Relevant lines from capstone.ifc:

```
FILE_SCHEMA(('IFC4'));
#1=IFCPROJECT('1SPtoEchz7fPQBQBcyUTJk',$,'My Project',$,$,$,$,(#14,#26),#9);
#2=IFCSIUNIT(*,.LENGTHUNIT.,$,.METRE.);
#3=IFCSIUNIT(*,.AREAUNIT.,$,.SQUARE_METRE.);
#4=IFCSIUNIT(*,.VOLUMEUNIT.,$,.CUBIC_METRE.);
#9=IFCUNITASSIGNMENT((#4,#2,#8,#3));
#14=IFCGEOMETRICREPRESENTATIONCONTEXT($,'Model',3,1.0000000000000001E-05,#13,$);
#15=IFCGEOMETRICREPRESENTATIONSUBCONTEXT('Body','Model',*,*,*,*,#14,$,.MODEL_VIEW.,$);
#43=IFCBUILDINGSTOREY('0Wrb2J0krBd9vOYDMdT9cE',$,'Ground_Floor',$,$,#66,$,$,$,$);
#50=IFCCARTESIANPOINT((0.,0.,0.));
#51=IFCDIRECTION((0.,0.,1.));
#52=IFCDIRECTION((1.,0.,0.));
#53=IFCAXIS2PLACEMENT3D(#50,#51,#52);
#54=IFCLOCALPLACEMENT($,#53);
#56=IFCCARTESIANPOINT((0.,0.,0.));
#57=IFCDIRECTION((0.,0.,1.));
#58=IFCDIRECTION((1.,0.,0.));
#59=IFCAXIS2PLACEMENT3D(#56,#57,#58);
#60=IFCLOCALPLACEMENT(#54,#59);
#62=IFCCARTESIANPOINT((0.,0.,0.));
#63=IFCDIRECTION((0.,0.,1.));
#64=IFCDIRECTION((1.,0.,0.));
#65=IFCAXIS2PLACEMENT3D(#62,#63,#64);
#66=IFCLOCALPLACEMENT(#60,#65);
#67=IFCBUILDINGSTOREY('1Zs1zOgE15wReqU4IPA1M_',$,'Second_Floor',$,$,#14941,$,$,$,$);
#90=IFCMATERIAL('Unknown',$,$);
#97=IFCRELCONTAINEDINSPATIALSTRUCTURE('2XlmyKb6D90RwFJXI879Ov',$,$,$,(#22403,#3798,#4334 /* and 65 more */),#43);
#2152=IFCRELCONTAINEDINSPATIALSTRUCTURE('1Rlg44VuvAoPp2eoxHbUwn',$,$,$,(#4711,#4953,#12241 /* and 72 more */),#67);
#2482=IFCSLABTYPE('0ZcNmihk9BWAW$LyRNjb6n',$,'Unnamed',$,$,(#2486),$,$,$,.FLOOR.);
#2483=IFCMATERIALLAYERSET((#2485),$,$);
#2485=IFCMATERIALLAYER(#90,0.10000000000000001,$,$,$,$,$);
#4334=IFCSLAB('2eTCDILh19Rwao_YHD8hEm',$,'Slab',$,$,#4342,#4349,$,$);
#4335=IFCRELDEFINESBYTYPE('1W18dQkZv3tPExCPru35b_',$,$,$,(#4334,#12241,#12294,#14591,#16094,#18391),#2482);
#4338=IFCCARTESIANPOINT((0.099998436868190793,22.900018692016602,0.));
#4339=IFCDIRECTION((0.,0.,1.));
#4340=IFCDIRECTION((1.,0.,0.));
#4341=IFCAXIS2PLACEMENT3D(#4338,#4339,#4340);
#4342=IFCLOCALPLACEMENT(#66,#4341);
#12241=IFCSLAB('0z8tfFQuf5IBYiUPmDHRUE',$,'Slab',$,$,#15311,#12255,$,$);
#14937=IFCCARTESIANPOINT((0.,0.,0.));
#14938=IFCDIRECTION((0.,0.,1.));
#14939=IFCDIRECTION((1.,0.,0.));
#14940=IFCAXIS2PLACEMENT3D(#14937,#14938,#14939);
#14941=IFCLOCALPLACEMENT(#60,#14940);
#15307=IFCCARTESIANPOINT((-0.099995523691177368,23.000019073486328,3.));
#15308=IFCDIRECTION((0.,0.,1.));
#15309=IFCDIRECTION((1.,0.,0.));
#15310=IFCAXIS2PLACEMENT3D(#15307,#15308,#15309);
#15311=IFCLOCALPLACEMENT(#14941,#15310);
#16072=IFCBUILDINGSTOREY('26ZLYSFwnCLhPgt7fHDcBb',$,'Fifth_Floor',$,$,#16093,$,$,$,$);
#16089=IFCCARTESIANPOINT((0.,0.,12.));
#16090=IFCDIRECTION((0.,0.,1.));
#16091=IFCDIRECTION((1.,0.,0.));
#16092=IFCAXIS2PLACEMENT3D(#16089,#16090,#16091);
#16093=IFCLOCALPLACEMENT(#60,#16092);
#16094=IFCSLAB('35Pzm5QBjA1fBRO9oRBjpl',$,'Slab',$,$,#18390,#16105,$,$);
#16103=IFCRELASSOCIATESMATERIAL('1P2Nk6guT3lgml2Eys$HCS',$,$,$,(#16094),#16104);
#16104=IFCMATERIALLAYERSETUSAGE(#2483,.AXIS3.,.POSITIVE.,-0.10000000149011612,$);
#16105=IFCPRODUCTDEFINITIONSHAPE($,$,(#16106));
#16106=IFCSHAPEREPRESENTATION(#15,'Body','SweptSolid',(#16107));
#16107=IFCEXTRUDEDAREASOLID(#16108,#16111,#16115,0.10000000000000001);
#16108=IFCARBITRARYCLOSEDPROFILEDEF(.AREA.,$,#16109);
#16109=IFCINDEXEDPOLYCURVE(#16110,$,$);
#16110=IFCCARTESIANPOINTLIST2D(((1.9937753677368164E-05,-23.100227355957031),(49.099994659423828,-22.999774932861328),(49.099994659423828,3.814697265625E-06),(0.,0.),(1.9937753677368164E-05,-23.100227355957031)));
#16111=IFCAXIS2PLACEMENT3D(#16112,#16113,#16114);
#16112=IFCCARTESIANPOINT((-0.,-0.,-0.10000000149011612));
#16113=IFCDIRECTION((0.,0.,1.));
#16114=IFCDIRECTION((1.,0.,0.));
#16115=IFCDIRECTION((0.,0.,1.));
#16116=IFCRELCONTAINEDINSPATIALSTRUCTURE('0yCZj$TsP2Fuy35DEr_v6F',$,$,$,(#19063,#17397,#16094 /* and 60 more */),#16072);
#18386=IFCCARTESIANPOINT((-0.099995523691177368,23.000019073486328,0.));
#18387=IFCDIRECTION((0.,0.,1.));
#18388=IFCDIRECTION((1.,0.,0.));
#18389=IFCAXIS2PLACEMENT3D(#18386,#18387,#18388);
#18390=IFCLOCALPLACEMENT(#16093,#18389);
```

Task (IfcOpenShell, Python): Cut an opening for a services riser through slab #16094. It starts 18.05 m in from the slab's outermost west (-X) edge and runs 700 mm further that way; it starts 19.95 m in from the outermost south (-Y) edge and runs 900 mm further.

```python
import numpy as np
import ifcopenshell
import ifcopenshell.api.feature
import ifcopenshell.api.geometry
import ifcopenshell.api.root
import ifcopenshell.geom
import ifcopenshell.util.placement
import ifcopenshell.util.representation
import ifcopenshell.util.shape
import ifcopenshell.util.unit

model = ifcopenshell.open("capstone.ifc")
unit_scale = ifcopenshell.util.unit.calculate_unit_scale(model)
settings = ifcopenshell.geom.settings()


def volume(element):
    """Net volume in cubic metres, openings subtracted."""
    shape = ifcopenshell.geom.create_shape(settings, element)
    return ifcopenshell.util.shape.get_volume(shape.geometry)


slab = model.by_id(16094)
before = volume(slab)

# Extent in the slab's own axes, in metres. The edges named are its -X and -Y sides.
slab_shape = ifcopenshell.geom.create_shape(settings, slab)
vertices = ifcopenshell.util.shape.get_vertices(slab_shape.geometry)
x_min, y_min, bottom = vertices.min(axis=0)
top = vertices[:, 2].max()

opening = ifcopenshell.api.root.create_entity(model, ifc_class="IfcOpeningElement", name="Services riser opening", predefined_type="OPENING")
context = ifcopenshell.util.representation.get_context(model, "Model", "Body", "MODEL_VIEW")
width, depth = 0.7, 0.9
outline = [(0.0, 0.0), (width, 0.0), (width, depth), (0.0, depth), (0.0, 0.0)]
# Overshoot both faces by 50 mm so the cut is clean.
shape = ifcopenshell.api.geometry.add_slab_representation(
    model, context=context, depth=top - bottom + 0.1, polyline=outline
)
ifcopenshell.api.geometry.assign_representation(model, product=opening, representation=shape)

matrix = ifcopenshell.util.placement.get_local_placement(slab.ObjectPlacement)
matrix[:, 3] = matrix @ np.append(np.array([x_min + 18.05, y_min + 19.95, bottom - 0.05]) / unit_scale, 1.0)
ifcopenshell.api.geometry.edit_object_placement(model, product=opening, matrix=matrix, is_si=False)
ifcopenshell.api.feature.add_feature(model, feature=opening, element=slab)

after = volume(slab)

print(f"slab volume {before:.3f} -> {after:.3f} m3")

model.write("capstone_updated.ifc")
```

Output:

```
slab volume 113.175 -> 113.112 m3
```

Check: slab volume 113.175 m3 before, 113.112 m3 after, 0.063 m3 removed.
